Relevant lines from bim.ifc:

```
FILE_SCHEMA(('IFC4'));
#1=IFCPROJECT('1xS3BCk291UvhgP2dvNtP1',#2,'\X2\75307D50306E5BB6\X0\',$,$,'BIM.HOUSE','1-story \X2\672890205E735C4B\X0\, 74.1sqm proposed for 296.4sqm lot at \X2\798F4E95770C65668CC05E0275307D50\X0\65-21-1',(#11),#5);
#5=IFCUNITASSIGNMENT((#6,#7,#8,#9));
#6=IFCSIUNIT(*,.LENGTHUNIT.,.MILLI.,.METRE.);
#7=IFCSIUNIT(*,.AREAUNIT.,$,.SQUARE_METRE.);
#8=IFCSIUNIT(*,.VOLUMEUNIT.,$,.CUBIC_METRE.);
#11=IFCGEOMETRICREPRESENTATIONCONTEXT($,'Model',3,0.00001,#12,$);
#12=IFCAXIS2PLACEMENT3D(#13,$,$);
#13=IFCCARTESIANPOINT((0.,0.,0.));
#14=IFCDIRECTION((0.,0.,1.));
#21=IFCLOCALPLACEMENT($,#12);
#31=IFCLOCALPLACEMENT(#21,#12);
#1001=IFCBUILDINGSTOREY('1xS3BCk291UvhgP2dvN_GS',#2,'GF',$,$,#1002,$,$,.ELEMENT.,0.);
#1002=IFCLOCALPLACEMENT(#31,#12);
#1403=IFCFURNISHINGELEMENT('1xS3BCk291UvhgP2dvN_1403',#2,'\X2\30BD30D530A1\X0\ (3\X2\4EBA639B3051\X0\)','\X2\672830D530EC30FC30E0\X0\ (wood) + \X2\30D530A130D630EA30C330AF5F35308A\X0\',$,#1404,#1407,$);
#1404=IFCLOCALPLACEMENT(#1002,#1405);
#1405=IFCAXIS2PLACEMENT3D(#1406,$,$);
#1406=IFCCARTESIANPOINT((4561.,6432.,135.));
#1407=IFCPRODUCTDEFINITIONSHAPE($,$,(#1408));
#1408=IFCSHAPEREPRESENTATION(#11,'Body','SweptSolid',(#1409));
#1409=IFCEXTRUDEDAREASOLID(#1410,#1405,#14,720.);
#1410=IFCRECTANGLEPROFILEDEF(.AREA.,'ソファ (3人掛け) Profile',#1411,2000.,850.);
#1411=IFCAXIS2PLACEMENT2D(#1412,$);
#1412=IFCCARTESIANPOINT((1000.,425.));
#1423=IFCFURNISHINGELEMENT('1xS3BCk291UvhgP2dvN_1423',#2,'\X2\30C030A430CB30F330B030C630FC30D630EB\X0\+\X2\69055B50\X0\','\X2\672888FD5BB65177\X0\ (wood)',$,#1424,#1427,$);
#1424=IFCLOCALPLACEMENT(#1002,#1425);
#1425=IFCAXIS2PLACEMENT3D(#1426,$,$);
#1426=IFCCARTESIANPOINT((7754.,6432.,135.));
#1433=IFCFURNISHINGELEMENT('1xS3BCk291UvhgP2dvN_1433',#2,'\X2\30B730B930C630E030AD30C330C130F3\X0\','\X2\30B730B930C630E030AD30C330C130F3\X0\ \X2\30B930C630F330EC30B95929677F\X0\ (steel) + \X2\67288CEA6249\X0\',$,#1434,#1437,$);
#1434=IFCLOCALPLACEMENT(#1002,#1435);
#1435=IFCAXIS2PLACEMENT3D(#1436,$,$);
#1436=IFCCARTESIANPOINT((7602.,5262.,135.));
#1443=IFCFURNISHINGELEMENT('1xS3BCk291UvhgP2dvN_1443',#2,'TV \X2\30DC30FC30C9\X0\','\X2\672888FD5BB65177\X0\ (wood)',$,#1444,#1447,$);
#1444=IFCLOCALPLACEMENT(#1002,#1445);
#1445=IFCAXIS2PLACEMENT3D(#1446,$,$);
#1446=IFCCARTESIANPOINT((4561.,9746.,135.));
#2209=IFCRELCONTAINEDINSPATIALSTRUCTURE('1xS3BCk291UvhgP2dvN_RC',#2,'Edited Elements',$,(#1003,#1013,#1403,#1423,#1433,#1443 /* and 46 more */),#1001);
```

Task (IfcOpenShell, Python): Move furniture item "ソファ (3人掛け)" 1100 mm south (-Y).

```python
import ifcopenshell
import ifcopenshell.api.geometry
import ifcopenshell.util.placement
import ifcopenshell.util.unit

model = ifcopenshell.open("bim.ifc")
unit_scale = ifcopenshell.util.unit.calculate_unit_scale(model)

item = model.by_id(1403)
matrix = ifcopenshell.util.placement.get_local_placement(item.ObjectPlacement)
matrix[1, 3] -= 1.1 / unit_scale
ifcopenshell.api.geometry.edit_object_placement(model, product=item, matrix=matrix, is_si=False)

print(ifcopenshell.util.placement.get_local_placement(item.ObjectPlacement).round(3) + 0.0)

model.write("bim-out.ifc")
```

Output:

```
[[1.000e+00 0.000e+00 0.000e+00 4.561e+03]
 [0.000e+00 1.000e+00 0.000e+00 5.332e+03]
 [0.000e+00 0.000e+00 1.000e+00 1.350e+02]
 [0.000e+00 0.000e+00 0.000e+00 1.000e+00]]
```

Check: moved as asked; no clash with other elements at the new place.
